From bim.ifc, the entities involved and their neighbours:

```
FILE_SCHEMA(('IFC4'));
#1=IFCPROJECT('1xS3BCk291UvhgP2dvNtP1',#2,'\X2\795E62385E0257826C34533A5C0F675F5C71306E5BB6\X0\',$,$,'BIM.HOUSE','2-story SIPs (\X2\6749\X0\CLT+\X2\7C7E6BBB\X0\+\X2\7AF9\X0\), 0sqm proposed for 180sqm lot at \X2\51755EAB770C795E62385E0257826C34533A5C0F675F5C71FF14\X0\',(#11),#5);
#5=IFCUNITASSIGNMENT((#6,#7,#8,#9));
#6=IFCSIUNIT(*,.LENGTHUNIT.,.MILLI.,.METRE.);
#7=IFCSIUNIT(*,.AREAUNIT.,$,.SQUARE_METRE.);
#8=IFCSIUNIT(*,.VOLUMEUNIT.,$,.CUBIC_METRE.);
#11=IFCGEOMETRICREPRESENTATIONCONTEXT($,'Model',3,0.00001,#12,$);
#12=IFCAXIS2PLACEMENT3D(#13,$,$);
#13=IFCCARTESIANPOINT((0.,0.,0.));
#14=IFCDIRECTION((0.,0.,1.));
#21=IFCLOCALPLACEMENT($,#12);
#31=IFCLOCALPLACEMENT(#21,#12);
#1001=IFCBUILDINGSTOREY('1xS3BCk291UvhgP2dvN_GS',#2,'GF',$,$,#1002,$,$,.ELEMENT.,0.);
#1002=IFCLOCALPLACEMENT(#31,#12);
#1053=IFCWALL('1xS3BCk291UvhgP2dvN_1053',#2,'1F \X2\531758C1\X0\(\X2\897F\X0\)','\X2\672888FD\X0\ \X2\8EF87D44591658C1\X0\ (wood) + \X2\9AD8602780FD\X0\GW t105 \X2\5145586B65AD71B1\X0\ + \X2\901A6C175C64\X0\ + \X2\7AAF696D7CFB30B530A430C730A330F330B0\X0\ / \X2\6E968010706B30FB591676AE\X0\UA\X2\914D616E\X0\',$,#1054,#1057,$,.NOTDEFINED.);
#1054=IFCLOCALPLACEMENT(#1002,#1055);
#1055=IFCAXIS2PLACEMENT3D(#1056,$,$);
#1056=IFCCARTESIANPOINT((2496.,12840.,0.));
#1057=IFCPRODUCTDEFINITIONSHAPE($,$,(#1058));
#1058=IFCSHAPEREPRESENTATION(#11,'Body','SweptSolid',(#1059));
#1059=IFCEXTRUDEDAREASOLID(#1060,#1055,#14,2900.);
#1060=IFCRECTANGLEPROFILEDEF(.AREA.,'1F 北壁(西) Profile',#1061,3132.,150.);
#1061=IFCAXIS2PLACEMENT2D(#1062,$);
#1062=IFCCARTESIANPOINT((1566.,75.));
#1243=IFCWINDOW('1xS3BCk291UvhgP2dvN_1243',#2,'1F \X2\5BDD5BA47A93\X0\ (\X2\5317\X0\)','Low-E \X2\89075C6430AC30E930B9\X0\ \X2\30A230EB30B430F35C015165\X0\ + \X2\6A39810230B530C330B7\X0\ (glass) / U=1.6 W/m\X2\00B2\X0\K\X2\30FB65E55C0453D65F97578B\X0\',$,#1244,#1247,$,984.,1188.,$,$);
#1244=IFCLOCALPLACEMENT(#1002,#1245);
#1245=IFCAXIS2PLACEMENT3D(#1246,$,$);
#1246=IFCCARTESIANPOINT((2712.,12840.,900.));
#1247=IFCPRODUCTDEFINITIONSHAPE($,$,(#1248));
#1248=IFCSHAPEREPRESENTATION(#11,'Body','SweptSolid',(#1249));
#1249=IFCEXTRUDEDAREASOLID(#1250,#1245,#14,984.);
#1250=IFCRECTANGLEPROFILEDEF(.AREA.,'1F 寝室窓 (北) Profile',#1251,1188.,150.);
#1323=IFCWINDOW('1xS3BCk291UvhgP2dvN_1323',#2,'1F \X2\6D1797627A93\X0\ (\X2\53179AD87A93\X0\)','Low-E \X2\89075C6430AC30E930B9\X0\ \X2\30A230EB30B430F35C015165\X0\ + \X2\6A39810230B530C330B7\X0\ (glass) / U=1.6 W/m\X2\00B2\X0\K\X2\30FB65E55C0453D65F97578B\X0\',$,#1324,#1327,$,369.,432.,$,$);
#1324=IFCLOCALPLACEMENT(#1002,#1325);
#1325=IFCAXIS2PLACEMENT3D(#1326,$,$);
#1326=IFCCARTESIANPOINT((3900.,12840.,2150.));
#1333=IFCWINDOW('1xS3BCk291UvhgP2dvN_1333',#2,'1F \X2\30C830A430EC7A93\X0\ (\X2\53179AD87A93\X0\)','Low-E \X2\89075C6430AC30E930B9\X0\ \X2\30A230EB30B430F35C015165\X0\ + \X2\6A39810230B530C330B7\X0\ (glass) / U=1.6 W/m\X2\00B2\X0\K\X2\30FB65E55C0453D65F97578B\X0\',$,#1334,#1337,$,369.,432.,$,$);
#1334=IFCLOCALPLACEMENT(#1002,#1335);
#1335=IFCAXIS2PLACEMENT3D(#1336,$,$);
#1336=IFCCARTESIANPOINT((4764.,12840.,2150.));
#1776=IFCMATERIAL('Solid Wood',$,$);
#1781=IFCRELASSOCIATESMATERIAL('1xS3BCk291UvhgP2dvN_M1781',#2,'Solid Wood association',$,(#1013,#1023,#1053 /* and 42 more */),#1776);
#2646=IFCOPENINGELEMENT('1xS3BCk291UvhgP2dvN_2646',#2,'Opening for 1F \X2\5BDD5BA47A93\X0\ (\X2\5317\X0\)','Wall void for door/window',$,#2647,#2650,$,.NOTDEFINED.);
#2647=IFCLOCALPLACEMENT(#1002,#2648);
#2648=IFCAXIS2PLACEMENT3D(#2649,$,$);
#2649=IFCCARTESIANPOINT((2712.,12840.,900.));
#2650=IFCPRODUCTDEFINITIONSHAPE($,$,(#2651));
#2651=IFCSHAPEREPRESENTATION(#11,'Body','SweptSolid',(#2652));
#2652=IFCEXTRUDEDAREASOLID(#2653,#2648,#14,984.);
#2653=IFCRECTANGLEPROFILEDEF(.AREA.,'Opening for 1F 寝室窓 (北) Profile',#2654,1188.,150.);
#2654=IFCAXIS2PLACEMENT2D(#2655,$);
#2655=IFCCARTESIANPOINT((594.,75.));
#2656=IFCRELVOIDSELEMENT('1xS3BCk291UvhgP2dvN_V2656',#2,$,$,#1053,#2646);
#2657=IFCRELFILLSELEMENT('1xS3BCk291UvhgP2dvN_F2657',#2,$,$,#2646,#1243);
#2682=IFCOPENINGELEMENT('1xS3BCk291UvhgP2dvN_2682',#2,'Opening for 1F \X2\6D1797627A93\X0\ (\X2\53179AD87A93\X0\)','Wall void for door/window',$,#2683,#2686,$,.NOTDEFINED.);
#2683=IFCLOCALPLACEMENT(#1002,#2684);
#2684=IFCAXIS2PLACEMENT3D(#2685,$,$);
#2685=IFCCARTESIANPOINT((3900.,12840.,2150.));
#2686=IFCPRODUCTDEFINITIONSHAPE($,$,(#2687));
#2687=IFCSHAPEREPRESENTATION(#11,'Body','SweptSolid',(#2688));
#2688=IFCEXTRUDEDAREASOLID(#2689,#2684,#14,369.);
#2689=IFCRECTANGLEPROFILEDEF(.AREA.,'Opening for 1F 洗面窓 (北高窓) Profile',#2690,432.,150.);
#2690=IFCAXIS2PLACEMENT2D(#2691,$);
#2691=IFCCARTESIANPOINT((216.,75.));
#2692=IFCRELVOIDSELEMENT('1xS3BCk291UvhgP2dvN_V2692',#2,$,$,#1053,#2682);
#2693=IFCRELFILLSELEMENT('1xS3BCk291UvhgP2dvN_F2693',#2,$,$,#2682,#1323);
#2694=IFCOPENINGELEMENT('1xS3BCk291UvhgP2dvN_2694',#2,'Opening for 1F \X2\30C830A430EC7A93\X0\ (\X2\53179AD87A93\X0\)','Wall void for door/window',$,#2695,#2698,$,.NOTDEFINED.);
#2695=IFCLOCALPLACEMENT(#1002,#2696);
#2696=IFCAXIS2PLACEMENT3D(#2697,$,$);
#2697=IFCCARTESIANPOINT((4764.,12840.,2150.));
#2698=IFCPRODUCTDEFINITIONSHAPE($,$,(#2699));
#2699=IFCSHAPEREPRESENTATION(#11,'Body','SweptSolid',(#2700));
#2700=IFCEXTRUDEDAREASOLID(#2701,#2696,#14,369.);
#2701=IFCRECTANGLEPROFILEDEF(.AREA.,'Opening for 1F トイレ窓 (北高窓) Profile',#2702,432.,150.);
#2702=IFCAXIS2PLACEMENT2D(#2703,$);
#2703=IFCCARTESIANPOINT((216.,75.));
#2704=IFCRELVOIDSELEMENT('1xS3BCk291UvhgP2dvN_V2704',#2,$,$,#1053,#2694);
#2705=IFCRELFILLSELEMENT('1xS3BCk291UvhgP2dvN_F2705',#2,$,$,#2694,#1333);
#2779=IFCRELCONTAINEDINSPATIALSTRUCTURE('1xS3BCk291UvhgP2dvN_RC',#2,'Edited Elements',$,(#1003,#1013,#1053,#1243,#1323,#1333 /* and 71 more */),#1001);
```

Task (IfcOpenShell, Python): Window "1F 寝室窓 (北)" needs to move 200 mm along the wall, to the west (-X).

```python
import ifcopenshell
import ifcopenshell.api.geometry
import ifcopenshell.util.placement

model = ifcopenshell.open("bim.ifc")

window = model.by_id(1243)
opening = window.FillsVoids[0].RelatingOpeningElement
wall = opening.VoidsElements[0].RelatingBuildingElement

wall_matrix = ifcopenshell.util.placement.get_local_placement(wall.ObjectPlacement)
shift = wall_matrix[:3, 0] * -200.0
before = ifcopenshell.util.placement.get_local_placement(window.ObjectPlacement)[:3, 3].copy()

# The window is not placed relative to its opening, so move both.
for product in (opening, window):
    matrix = ifcopenshell.util.placement.get_local_placement(product.ObjectPlacement)
    matrix[:3, 3] += shift
    ifcopenshell.api.geometry.edit_object_placement(model, product=product, matrix=matrix, is_si=False)

after = ifcopenshell.util.placement.get_local_placement(window.ObjectPlacement)[:3, 3]
print("window moved by", (after - before).round(3) + 0.0)

model.write("bim_edited.ifc")
```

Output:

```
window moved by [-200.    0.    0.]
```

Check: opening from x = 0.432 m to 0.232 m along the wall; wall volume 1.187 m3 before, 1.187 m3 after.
